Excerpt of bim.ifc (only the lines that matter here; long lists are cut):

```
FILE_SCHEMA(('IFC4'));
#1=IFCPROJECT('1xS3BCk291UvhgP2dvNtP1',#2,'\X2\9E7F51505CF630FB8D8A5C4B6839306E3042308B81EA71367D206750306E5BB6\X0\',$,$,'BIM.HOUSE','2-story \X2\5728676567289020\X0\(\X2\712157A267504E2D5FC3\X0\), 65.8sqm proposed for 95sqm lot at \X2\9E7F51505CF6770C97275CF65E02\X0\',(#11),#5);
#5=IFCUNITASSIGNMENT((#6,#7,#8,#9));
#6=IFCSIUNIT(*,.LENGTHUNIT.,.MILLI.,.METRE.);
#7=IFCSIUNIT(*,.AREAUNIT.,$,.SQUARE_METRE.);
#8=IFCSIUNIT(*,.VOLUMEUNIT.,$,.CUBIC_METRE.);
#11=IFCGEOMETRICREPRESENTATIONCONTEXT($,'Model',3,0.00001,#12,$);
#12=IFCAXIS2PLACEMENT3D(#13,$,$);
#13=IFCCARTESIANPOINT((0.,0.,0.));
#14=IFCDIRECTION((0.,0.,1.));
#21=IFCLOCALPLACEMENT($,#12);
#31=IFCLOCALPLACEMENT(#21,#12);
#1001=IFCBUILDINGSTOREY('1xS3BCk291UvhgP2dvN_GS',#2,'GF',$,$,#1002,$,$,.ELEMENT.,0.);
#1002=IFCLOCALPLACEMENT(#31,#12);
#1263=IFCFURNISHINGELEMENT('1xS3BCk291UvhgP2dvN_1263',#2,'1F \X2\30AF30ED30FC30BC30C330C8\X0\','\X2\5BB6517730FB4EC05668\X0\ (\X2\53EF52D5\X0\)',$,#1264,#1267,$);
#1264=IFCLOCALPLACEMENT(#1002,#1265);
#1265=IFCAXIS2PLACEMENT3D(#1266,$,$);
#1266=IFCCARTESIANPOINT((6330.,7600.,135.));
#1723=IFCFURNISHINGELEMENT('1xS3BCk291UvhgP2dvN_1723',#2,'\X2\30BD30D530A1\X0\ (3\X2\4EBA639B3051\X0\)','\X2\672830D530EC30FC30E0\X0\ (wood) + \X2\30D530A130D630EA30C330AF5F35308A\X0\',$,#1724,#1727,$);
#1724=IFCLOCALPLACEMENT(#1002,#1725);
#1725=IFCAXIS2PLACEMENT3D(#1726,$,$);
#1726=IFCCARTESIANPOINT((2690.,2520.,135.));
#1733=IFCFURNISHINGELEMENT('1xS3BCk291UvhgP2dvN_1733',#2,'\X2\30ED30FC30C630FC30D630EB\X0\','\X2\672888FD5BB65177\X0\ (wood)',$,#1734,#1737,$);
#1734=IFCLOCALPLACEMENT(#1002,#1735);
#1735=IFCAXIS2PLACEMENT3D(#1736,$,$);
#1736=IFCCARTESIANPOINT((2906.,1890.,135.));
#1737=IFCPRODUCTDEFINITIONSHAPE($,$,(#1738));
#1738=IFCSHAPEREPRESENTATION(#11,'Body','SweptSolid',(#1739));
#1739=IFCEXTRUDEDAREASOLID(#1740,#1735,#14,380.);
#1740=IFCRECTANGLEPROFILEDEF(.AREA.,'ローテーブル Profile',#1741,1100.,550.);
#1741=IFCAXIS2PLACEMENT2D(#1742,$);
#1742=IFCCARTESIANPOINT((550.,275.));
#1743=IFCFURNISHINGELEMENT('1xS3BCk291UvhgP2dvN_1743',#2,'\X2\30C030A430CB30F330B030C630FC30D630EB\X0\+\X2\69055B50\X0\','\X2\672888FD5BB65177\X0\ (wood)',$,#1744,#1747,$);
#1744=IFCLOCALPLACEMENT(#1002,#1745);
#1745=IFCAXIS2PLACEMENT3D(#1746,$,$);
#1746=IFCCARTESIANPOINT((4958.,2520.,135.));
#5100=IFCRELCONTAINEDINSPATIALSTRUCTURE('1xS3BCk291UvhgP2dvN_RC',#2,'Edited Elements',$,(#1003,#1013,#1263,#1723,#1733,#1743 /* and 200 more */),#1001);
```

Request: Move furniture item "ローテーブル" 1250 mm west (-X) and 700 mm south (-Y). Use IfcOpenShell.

```python
import ifcopenshell
import ifcopenshell.api.geometry
import ifcopenshell.util.placement

model = ifcopenshell.open("bim.ifc")

item = model.by_id(1733)
matrix = ifcopenshell.util.placement.get_local_placement(item.ObjectPlacement)
matrix[0, 3] -= 1250.0
matrix[1, 3] -= 700.0
ifcopenshell.api.geometry.edit_object_placement(model, product=item, matrix=matrix, is_si=False)

print(ifcopenshell.util.placement.get_local_placement(item.ObjectPlacement).round(3) + 0.0)

model.write("bim-out.ifc")
```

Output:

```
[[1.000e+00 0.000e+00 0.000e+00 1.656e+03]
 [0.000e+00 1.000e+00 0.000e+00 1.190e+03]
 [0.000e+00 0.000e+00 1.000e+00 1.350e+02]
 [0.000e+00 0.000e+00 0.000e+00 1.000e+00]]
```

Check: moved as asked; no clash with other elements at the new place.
